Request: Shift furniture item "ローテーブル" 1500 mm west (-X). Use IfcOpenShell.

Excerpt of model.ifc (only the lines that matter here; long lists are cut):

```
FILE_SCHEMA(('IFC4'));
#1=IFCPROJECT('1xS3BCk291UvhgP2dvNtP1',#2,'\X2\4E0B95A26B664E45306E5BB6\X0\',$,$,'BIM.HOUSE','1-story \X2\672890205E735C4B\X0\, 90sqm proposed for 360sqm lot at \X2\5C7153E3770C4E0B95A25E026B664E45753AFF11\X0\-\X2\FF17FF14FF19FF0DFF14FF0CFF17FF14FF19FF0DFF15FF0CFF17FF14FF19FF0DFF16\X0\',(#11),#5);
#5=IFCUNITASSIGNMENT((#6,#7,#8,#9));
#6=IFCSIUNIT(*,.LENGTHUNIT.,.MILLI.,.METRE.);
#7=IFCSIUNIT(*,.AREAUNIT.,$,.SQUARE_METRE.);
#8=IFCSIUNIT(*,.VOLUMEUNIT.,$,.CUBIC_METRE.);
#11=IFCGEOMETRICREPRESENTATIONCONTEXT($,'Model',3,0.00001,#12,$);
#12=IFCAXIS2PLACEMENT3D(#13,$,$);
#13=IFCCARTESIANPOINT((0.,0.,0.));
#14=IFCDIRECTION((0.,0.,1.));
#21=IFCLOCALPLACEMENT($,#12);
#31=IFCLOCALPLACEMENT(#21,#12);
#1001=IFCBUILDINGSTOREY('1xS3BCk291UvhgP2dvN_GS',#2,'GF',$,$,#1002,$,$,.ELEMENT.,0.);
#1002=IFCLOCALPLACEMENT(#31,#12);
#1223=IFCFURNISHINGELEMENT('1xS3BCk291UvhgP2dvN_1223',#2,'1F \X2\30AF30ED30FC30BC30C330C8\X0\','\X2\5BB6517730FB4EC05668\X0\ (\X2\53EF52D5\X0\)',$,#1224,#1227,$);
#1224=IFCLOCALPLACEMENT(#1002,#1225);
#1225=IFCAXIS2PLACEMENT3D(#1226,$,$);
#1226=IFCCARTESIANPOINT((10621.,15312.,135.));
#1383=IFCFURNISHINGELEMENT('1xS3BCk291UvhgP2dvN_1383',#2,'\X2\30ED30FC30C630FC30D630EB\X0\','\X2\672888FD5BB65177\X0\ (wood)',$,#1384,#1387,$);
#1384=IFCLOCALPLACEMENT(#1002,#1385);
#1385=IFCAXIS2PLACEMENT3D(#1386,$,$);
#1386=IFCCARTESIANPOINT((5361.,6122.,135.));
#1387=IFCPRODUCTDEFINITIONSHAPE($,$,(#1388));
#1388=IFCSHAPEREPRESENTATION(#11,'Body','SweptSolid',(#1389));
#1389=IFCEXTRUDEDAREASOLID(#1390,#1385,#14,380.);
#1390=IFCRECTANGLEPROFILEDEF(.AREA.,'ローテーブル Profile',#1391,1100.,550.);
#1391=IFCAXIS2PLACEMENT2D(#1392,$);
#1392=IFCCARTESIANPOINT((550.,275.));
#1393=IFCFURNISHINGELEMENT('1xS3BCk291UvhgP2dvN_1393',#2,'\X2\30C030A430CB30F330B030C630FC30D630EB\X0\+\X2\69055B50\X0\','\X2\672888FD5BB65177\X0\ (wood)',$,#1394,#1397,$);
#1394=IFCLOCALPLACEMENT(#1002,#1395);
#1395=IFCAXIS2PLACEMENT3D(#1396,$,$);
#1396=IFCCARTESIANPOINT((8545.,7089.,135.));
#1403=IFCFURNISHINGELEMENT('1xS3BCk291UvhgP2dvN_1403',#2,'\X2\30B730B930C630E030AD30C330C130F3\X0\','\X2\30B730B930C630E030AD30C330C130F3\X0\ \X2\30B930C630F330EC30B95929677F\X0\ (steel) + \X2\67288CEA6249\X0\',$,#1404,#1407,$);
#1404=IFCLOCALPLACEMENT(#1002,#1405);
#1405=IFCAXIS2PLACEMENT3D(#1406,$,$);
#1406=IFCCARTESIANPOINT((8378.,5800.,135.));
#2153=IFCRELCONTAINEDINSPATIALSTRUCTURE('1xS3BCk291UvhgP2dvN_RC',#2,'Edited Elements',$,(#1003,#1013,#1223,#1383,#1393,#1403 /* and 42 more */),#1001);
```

```python
import ifcopenshell
import ifcopenshell.api.geometry
import ifcopenshell.util.placement
import ifcopenshell.util.unit

model = ifcopenshell.open("model.ifc")
unit_scale = ifcopenshell.util.unit.calculate_unit_scale(model)

item = model.by_guid("1xS3BCk291UvhgP2dvN_1383")
matrix = ifcopenshell.util.placement.get_local_placement(item.ObjectPlacement)
matrix[0, 3] -= 1.5 / unit_scale
ifcopenshell.api.geometry.edit_object_placement(model, product=item, matrix=matrix, is_si=False)

print(ifcopenshell.util.placement.get_local_placement(item.ObjectPlacement).round(3) + 0.0)

model.write("model_v2.ifc")
```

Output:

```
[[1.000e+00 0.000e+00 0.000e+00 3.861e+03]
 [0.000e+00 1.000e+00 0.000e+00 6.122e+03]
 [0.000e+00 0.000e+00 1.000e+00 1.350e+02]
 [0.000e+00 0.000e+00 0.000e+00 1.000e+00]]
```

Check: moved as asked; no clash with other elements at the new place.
